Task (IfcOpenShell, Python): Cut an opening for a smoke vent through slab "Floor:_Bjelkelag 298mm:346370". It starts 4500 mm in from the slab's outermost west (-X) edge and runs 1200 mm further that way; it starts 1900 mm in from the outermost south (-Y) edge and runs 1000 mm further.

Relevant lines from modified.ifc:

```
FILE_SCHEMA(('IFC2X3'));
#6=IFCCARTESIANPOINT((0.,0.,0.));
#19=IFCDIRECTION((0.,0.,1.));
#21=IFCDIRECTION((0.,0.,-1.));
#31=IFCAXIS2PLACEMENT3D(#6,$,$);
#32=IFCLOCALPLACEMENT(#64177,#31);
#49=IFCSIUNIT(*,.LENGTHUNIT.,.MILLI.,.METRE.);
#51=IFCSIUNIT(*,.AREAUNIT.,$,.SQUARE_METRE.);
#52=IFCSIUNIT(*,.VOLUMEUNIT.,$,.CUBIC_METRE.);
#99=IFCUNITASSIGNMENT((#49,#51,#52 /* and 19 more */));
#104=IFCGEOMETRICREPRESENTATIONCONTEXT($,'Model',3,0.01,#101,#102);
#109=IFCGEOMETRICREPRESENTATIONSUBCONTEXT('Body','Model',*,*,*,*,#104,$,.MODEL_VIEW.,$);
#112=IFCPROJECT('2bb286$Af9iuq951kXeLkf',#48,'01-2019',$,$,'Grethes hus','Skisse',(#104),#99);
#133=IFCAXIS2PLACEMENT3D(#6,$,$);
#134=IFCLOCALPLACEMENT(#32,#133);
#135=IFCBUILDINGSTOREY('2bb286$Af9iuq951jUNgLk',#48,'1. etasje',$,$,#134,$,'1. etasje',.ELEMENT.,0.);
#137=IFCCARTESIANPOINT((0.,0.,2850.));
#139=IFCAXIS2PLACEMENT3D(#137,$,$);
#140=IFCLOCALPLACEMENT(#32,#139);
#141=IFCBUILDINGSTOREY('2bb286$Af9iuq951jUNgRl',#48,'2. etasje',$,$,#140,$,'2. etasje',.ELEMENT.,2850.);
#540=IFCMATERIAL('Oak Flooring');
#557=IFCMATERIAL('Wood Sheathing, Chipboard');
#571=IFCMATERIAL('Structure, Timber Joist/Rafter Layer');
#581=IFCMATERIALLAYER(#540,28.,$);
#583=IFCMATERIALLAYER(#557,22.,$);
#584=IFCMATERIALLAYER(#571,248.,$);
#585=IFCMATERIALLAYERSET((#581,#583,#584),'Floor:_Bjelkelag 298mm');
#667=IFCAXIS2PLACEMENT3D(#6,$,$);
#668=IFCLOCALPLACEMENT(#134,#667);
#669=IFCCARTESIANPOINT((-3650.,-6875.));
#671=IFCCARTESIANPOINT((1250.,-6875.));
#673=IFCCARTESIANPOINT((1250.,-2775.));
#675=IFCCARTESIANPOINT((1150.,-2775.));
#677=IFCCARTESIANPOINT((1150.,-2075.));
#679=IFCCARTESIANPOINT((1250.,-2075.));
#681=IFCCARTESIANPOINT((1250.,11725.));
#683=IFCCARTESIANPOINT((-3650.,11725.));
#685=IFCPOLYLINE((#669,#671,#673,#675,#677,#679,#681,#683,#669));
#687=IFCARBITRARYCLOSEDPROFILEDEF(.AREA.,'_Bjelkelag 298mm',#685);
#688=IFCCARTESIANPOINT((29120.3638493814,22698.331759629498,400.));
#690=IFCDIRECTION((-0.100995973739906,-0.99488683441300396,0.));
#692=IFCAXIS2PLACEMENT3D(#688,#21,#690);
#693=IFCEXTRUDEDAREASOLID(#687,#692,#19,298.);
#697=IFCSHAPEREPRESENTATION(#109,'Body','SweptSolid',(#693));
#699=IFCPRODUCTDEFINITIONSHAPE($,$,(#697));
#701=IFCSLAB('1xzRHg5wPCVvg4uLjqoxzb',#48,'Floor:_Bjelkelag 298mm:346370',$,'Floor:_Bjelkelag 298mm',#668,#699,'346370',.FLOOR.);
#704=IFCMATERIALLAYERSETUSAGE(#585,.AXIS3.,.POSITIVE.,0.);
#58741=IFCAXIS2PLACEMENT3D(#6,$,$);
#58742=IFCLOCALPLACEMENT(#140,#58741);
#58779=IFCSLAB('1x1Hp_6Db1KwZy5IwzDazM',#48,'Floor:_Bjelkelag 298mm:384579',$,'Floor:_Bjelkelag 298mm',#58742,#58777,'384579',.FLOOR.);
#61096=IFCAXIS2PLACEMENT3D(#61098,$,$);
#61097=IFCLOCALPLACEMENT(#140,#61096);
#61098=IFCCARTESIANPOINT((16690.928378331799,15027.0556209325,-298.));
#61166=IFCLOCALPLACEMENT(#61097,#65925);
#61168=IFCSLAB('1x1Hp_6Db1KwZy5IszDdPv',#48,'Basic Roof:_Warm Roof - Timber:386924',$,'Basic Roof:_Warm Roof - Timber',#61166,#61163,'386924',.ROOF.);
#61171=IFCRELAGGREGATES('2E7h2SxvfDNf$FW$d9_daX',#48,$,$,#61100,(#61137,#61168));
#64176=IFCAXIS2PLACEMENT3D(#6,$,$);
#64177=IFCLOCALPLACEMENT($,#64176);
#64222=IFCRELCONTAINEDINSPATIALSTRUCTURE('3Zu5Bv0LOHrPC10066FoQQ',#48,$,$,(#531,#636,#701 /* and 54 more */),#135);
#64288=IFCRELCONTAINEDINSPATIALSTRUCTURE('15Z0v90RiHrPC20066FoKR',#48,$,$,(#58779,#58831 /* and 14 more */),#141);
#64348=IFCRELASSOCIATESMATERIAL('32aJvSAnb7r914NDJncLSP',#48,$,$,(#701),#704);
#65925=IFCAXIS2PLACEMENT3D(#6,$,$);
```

```python
import numpy as np
import ifcopenshell
import ifcopenshell.api.feature
import ifcopenshell.api.geometry
import ifcopenshell.api.root
import ifcopenshell.geom
import ifcopenshell.util.placement
import ifcopenshell.util.representation
import ifcopenshell.util.shape
import ifcopenshell.util.unit

model = ifcopenshell.open("modified.ifc")
unit_scale = ifcopenshell.util.unit.calculate_unit_scale(model)
settings = ifcopenshell.geom.settings()


def volume(element):
    """Net volume in cubic metres, openings subtracted."""
    shape = ifcopenshell.geom.create_shape(settings, element)
    return ifcopenshell.util.shape.get_volume(shape.geometry)


slab = model.by_guid("1xzRHg5wPCVvg4uLjqoxzb")
before = volume(slab)

# Extent in the slab's own axes, in metres. The edges named are its -X and -Y sides.
slab_shape = ifcopenshell.geom.create_shape(settings, slab)
vertices = ifcopenshell.util.shape.get_vertices(slab_shape.geometry)
x_min, y_min, bottom = vertices.min(axis=0)
top = vertices[:, 2].max()

opening = ifcopenshell.api.root.create_entity(model, ifc_class="IfcOpeningElement", name="Smoke vent opening")
context = ifcopenshell.util.representation.get_context(model, "Model", "Body", "MODEL_VIEW")
width, depth = 1.2, 1
outline = [(0.0, 0.0), (width, 0.0), (width, depth), (0.0, depth), (0.0, 0.0)]
# Overshoot both faces by 50 mm so the cut is clean.
shape = ifcopenshell.api.geometry.add_slab_representation(
    model, context=context, depth=top - bottom + 0.1, polyline=outline
)
ifcopenshell.api.geometry.assign_representation(model, product=opening, representation=shape)

matrix = ifcopenshell.util.placement.get_local_placement(slab.ObjectPlacement)
matrix[:, 3] = matrix @ np.append(np.array([x_min + 4.5, y_min + 1.9, bottom - 0.05]) / unit_scale, 1.0)
ifcopenshell.api.geometry.edit_object_placement(model, product=opening, matrix=matrix, is_si=False)
ifcopenshell.api.feature.add_feature(model, feature=opening, element=slab)

after = volume(slab)

print(f"slab volume {before:.3f} -> {after:.3f} m3")

model.write("modified_v2.ifc")
```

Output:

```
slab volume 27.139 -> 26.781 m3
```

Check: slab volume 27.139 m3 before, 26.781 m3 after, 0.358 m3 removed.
